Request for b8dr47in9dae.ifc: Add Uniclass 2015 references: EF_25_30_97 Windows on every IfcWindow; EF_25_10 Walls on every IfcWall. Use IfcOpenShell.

First a look at what the model holds.

```python
import ifcopenshell

model = ifcopenshell.open("b8dr47in9dae.ifc")
print(model.schema)
print("classifications:", [c.Name for c in model.by_type("IfcClassification")])
for ifc_class in ("IfcDoor", "IfcRoof", "IfcStair", "IfcWall", "IfcWindow"):
    print(ifc_class, len(model.by_type(ifc_class)))
```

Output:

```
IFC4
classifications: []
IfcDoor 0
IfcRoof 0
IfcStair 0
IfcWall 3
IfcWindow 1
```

```python
import ifcopenshell
import ifcopenshell.api.classification

model = ifcopenshell.open("b8dr47in9dae.ifc")

system = ifcopenshell.api.classification.add_classification(model, classification="Uniclass 2015")

codes = {
    "IfcWindow": ("EF_25_30_97", "Windows"),
    "IfcWall": ("EF_25_10", "Walls"),
}
for ifc_class, (code, name) in codes.items():
    products = model.by_type(ifc_class)
    ifcopenshell.api.classification.add_reference(
        model, products=products, classification=system, identification=code, name=name
    )
    print(code, len(products))

model.write("b8dr47in9dae_edited.ifc")
```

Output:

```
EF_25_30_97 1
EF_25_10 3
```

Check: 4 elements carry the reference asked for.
